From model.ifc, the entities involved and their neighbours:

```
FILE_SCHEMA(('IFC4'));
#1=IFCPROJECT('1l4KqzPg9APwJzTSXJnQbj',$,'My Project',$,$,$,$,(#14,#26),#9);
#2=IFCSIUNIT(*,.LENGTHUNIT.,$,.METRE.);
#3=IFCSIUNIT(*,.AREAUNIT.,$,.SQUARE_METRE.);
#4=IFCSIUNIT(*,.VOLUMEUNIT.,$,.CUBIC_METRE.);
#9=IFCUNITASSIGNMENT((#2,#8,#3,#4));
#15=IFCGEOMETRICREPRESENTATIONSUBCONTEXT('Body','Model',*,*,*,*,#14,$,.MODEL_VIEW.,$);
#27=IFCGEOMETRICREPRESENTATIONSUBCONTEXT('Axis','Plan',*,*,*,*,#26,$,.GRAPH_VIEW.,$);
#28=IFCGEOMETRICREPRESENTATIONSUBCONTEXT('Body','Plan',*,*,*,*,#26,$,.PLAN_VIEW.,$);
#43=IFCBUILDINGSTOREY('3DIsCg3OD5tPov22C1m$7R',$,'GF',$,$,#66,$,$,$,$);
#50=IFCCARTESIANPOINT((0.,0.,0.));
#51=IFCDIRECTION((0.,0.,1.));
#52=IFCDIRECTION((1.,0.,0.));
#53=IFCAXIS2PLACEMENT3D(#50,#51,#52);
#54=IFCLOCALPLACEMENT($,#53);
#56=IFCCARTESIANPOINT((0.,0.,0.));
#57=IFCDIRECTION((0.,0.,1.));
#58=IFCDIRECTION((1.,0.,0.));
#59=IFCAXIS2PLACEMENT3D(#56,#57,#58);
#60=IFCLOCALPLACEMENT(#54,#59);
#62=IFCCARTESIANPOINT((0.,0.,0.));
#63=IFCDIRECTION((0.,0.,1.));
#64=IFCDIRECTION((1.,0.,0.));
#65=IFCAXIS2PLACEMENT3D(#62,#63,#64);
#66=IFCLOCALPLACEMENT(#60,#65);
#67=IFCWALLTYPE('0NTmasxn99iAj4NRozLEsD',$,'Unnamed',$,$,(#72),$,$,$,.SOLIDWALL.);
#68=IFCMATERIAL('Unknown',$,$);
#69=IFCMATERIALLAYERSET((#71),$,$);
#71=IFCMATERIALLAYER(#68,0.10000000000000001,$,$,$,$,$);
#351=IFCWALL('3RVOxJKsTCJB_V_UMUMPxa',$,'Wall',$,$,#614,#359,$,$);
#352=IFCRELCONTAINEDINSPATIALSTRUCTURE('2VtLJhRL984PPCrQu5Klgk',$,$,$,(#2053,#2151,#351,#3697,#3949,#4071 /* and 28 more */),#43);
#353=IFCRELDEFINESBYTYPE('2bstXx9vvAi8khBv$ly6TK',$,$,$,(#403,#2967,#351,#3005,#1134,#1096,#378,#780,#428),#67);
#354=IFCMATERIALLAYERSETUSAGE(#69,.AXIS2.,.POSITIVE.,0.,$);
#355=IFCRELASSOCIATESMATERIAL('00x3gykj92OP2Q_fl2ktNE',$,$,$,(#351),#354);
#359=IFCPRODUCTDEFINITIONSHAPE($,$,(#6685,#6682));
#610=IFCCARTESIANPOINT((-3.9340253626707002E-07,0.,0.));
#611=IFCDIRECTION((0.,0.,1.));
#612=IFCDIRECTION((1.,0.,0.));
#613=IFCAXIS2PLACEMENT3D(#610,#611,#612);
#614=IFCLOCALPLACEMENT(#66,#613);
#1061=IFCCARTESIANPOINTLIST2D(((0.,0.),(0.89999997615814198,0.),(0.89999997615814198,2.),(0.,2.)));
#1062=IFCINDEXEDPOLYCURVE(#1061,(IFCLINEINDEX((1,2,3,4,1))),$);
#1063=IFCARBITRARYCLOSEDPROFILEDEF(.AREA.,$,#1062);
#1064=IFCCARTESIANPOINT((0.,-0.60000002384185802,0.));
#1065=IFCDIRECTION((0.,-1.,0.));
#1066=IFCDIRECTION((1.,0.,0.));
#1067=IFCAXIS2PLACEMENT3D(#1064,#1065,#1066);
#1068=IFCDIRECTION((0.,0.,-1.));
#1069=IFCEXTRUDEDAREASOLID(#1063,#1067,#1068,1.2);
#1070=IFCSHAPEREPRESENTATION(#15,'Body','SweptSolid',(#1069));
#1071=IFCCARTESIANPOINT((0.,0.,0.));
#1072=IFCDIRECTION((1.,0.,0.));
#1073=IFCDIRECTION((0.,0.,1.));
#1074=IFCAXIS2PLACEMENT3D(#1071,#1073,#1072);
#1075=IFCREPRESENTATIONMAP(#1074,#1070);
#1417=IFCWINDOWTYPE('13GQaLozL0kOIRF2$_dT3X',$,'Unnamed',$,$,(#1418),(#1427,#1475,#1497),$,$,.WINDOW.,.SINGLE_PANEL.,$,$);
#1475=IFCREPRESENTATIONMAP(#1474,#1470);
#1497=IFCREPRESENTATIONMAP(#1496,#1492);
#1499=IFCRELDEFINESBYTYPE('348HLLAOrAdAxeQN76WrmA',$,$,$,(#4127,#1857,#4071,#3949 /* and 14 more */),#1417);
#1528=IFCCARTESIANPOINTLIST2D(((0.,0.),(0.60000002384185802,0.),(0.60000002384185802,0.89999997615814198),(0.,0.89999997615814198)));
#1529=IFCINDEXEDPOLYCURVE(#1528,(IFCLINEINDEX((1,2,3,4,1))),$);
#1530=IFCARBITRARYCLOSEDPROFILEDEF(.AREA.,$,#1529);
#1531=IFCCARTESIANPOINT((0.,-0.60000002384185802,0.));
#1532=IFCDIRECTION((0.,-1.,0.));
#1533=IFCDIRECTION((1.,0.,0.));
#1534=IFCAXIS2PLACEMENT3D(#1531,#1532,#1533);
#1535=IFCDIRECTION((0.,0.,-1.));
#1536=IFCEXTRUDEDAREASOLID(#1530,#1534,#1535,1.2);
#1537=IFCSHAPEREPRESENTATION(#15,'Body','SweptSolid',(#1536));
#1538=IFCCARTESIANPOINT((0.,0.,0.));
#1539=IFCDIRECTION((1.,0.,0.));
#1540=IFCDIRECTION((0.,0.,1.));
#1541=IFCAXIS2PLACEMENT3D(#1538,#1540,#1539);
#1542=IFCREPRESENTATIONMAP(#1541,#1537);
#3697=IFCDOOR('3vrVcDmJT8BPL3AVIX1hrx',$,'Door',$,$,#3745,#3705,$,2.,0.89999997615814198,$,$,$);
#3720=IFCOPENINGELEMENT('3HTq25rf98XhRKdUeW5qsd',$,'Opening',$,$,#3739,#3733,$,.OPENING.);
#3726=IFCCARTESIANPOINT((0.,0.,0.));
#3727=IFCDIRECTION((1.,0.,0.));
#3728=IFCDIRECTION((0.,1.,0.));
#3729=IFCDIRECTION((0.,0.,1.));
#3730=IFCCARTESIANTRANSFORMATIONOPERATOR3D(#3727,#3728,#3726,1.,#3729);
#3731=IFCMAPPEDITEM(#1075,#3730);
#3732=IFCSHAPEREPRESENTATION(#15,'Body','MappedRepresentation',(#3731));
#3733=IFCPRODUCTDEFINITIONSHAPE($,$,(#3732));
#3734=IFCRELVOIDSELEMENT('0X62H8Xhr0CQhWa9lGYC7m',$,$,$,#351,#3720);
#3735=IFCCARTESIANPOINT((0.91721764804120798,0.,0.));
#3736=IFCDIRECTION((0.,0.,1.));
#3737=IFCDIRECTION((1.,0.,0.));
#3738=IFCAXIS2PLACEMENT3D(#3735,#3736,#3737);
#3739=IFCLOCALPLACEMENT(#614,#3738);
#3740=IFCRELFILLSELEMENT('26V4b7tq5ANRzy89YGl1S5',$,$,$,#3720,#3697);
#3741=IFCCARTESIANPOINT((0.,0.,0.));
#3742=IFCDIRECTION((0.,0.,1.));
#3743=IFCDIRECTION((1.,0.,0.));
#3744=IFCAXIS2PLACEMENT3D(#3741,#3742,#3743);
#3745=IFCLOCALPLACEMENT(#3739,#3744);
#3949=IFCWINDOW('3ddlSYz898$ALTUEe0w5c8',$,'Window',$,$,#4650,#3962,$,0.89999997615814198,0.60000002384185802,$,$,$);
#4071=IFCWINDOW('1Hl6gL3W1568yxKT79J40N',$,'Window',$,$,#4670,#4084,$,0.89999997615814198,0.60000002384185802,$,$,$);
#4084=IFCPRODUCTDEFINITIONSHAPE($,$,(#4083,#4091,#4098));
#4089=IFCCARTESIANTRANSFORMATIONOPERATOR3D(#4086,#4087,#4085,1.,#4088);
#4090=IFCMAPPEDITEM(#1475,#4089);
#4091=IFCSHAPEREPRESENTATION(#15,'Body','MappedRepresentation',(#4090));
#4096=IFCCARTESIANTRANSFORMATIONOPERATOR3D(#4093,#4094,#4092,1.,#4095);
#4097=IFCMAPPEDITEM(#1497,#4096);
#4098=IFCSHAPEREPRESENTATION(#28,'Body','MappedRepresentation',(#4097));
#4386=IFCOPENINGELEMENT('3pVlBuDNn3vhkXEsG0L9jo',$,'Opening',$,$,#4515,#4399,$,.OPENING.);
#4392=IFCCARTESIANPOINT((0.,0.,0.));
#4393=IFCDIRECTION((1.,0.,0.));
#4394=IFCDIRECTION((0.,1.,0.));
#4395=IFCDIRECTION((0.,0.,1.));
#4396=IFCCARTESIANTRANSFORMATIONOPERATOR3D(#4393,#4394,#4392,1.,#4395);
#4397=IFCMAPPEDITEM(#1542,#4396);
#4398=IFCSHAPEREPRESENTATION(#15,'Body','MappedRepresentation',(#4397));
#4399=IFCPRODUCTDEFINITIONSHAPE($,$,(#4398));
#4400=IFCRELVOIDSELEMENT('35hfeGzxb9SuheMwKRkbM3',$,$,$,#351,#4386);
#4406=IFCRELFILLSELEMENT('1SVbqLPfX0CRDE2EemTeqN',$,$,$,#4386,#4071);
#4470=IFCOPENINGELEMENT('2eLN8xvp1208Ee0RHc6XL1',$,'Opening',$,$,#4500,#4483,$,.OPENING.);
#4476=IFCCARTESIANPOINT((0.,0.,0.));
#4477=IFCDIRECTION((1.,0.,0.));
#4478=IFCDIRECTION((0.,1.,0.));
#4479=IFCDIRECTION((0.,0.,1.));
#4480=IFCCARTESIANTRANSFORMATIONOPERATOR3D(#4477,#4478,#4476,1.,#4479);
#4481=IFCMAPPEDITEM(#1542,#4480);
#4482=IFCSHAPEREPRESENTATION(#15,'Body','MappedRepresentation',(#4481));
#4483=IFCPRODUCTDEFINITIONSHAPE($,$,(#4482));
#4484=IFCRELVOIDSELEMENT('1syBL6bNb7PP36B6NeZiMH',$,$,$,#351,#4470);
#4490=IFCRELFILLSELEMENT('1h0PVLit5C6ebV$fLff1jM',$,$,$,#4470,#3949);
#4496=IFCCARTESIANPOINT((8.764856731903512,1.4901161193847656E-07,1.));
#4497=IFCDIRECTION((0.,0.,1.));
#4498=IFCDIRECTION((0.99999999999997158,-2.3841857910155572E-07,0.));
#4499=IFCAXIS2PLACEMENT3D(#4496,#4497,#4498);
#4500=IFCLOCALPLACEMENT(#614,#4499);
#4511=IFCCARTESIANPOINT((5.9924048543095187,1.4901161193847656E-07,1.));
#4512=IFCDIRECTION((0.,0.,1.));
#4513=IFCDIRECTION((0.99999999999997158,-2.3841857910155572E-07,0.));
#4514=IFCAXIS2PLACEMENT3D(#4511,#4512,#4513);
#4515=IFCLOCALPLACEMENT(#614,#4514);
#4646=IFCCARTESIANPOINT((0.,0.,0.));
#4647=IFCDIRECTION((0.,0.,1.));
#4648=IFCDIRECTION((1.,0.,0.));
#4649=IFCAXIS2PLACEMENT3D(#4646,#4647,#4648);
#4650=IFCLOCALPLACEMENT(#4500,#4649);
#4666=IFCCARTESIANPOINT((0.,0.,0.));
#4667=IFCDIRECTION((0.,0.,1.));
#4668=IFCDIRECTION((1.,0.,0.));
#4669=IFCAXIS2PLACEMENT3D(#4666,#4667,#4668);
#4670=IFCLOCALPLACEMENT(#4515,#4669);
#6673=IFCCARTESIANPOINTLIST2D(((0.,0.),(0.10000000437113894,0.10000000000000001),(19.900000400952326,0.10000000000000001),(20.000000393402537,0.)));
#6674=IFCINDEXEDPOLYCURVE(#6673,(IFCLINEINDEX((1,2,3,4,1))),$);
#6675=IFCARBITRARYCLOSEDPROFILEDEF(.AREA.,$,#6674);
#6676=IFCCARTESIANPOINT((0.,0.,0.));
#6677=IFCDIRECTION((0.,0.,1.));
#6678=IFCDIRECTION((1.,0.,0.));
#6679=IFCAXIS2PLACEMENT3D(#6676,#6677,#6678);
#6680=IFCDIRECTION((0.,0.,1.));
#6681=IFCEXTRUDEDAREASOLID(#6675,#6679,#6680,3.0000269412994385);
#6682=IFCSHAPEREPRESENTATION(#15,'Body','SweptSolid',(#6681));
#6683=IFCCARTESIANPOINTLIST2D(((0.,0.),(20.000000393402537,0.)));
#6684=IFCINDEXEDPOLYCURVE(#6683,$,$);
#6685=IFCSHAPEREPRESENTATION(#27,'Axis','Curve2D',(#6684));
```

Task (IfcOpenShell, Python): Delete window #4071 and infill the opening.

```python
import ifcopenshell
import ifcopenshell.api.feature
import ifcopenshell.api.root
import ifcopenshell.geom
import ifcopenshell.util.shape

model = ifcopenshell.open("model.ifc")
settings = ifcopenshell.geom.settings()


def volume(element):
    """Net volume in cubic metres, openings subtracted."""
    shape = ifcopenshell.geom.create_shape(settings, element)
    return ifcopenshell.util.shape.get_volume(shape.geometry)


window = model.by_guid("1Hl6gL3W1568yxKT79J40N")
opening = window.FillsVoids[0].RelatingOpeningElement
wall = opening.VoidsElements[0].RelatingBuildingElement
before = volume(wall)

ifcopenshell.api.root.remove_product(model, product=window)
ifcopenshell.api.feature.remove_feature(model, feature=opening)

after = volume(wall)

print(f"wall volume {before:.3f} -> {after:.3f} m3")

model.write("model_updated.ifc")
```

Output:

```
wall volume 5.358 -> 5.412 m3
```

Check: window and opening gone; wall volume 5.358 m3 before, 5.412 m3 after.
